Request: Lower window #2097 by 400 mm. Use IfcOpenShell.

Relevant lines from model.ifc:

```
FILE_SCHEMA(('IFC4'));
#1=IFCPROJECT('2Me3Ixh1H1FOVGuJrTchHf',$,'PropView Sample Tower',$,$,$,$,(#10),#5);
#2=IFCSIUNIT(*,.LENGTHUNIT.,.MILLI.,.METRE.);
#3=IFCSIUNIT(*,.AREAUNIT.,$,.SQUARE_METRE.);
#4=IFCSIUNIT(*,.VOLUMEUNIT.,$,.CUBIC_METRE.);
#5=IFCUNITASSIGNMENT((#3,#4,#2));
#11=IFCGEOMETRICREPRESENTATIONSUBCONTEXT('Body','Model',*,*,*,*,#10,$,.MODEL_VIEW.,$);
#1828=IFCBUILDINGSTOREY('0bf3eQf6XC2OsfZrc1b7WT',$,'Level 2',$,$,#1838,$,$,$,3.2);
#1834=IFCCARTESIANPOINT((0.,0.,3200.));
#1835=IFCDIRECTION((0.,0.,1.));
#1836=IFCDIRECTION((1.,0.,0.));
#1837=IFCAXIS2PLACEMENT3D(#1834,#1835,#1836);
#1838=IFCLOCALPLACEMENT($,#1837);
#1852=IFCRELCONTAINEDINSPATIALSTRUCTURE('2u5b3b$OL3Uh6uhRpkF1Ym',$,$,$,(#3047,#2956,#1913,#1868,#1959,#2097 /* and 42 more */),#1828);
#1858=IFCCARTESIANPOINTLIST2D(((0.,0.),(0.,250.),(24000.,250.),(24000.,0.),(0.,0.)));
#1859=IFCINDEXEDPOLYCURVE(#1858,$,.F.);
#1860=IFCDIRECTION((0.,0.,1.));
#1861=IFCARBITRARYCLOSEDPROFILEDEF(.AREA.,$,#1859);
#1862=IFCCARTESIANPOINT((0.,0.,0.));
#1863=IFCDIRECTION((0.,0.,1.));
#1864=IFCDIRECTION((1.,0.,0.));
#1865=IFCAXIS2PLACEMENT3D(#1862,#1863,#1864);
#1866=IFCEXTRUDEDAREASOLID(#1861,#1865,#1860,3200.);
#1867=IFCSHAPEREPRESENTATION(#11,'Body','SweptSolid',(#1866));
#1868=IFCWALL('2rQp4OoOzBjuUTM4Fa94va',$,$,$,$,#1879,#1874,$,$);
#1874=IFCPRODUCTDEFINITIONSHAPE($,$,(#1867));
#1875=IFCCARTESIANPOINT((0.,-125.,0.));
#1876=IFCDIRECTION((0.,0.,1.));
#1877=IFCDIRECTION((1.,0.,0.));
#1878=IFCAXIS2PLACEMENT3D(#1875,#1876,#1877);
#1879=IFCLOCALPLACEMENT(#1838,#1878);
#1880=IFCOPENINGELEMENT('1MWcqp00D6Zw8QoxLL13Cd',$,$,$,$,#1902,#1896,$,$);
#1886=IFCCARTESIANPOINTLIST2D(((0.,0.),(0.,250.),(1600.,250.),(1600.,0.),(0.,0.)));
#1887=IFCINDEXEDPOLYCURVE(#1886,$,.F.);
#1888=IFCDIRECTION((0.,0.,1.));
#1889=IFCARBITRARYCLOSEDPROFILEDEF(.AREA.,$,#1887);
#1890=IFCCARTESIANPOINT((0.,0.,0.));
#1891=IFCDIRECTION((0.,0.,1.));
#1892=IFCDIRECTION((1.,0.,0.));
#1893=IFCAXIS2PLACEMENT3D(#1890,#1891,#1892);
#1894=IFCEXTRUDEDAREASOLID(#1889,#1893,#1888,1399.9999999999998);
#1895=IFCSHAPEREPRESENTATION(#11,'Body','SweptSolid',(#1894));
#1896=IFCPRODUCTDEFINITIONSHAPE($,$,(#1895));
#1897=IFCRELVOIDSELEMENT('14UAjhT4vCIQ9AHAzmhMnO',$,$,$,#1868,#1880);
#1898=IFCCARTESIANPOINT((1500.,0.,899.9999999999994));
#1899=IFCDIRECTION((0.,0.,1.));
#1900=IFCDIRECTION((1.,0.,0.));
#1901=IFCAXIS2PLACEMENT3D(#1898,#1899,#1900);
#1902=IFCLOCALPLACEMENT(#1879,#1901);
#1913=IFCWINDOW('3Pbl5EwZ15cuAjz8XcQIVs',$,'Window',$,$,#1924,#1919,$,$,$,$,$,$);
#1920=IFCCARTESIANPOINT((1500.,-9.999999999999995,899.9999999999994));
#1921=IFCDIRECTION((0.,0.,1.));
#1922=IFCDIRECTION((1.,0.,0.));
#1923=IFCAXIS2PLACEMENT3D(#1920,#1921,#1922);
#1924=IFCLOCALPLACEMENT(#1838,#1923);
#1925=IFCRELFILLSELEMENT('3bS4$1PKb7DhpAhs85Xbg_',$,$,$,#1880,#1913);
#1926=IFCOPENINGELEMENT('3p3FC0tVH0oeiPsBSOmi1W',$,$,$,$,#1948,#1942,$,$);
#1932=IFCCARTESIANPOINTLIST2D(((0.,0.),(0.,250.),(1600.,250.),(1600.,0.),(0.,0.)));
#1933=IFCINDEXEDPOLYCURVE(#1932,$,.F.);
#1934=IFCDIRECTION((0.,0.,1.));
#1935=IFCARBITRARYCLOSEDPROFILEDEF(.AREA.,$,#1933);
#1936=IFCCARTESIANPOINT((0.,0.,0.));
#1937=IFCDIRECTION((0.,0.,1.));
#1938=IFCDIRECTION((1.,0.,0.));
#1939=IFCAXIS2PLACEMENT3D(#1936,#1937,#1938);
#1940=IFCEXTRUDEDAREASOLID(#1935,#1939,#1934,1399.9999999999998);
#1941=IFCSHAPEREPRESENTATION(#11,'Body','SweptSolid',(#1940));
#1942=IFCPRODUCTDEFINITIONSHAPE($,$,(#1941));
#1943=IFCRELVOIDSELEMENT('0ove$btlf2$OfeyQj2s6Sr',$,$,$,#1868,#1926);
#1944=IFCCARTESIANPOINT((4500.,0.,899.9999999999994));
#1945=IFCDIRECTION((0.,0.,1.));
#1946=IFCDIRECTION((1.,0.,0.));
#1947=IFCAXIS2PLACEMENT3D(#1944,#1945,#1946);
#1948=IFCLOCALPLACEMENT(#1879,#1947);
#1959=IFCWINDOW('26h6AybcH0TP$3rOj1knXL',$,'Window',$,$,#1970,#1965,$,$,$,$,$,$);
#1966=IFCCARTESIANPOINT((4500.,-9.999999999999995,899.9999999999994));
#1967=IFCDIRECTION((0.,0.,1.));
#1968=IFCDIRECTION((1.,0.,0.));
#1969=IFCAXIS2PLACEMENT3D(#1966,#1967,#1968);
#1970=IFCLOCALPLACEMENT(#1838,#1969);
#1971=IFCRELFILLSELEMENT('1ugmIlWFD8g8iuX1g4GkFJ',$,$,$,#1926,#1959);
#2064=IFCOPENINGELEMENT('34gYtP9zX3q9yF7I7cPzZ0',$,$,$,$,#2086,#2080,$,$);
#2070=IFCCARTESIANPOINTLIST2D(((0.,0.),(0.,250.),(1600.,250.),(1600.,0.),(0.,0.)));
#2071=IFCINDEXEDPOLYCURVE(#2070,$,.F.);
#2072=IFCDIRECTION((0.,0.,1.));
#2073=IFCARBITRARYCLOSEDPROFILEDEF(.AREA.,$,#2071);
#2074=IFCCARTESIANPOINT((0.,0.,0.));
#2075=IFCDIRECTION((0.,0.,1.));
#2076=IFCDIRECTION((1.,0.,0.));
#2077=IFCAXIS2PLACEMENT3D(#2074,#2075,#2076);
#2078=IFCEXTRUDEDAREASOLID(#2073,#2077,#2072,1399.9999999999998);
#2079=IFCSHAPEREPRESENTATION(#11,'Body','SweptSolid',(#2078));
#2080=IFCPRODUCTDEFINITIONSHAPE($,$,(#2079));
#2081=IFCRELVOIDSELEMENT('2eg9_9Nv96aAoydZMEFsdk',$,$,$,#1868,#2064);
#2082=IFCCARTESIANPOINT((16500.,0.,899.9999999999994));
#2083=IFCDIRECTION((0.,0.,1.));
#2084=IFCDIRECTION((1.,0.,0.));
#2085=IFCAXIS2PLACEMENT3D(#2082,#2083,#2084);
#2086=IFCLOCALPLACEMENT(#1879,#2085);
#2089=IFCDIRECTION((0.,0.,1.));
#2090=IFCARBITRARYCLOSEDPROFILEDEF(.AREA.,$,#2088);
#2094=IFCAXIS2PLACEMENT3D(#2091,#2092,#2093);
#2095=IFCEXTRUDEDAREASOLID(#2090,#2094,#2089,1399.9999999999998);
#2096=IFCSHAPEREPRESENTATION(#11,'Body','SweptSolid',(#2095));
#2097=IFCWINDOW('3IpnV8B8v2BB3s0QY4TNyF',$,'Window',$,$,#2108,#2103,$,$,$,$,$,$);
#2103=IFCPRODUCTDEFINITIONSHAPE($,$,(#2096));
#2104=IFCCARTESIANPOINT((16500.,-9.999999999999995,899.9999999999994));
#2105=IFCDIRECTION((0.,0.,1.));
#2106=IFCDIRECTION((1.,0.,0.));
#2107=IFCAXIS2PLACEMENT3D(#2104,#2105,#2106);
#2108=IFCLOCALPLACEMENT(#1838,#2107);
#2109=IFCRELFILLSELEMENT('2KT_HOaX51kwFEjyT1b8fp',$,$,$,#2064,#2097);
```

```python
import numpy as np
import ifcopenshell
import ifcopenshell.api.geometry
import ifcopenshell.util.placement
import ifcopenshell.util.unit

model = ifcopenshell.open("model.ifc")
unit_scale = ifcopenshell.util.unit.calculate_unit_scale(model)

window = model.by_id(2097)
opening = window.FillsVoids[0].RelatingOpeningElement
dz = -0.4 / unit_scale

shift = np.array([0.0, 0.0, dz])
# The window is not placed relative to its opening, so move both.
for product in (opening, window):
    matrix = ifcopenshell.util.placement.get_local_placement(product.ObjectPlacement)
    matrix[:3, 3] += shift
    ifcopenshell.api.geometry.edit_object_placement(model, product=product, matrix=matrix, is_si=False)

print(f"moved by {dz * unit_scale:+.3f} m")

model.write("model_edited.ifc")
```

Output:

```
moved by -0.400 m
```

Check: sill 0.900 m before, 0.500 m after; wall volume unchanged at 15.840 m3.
